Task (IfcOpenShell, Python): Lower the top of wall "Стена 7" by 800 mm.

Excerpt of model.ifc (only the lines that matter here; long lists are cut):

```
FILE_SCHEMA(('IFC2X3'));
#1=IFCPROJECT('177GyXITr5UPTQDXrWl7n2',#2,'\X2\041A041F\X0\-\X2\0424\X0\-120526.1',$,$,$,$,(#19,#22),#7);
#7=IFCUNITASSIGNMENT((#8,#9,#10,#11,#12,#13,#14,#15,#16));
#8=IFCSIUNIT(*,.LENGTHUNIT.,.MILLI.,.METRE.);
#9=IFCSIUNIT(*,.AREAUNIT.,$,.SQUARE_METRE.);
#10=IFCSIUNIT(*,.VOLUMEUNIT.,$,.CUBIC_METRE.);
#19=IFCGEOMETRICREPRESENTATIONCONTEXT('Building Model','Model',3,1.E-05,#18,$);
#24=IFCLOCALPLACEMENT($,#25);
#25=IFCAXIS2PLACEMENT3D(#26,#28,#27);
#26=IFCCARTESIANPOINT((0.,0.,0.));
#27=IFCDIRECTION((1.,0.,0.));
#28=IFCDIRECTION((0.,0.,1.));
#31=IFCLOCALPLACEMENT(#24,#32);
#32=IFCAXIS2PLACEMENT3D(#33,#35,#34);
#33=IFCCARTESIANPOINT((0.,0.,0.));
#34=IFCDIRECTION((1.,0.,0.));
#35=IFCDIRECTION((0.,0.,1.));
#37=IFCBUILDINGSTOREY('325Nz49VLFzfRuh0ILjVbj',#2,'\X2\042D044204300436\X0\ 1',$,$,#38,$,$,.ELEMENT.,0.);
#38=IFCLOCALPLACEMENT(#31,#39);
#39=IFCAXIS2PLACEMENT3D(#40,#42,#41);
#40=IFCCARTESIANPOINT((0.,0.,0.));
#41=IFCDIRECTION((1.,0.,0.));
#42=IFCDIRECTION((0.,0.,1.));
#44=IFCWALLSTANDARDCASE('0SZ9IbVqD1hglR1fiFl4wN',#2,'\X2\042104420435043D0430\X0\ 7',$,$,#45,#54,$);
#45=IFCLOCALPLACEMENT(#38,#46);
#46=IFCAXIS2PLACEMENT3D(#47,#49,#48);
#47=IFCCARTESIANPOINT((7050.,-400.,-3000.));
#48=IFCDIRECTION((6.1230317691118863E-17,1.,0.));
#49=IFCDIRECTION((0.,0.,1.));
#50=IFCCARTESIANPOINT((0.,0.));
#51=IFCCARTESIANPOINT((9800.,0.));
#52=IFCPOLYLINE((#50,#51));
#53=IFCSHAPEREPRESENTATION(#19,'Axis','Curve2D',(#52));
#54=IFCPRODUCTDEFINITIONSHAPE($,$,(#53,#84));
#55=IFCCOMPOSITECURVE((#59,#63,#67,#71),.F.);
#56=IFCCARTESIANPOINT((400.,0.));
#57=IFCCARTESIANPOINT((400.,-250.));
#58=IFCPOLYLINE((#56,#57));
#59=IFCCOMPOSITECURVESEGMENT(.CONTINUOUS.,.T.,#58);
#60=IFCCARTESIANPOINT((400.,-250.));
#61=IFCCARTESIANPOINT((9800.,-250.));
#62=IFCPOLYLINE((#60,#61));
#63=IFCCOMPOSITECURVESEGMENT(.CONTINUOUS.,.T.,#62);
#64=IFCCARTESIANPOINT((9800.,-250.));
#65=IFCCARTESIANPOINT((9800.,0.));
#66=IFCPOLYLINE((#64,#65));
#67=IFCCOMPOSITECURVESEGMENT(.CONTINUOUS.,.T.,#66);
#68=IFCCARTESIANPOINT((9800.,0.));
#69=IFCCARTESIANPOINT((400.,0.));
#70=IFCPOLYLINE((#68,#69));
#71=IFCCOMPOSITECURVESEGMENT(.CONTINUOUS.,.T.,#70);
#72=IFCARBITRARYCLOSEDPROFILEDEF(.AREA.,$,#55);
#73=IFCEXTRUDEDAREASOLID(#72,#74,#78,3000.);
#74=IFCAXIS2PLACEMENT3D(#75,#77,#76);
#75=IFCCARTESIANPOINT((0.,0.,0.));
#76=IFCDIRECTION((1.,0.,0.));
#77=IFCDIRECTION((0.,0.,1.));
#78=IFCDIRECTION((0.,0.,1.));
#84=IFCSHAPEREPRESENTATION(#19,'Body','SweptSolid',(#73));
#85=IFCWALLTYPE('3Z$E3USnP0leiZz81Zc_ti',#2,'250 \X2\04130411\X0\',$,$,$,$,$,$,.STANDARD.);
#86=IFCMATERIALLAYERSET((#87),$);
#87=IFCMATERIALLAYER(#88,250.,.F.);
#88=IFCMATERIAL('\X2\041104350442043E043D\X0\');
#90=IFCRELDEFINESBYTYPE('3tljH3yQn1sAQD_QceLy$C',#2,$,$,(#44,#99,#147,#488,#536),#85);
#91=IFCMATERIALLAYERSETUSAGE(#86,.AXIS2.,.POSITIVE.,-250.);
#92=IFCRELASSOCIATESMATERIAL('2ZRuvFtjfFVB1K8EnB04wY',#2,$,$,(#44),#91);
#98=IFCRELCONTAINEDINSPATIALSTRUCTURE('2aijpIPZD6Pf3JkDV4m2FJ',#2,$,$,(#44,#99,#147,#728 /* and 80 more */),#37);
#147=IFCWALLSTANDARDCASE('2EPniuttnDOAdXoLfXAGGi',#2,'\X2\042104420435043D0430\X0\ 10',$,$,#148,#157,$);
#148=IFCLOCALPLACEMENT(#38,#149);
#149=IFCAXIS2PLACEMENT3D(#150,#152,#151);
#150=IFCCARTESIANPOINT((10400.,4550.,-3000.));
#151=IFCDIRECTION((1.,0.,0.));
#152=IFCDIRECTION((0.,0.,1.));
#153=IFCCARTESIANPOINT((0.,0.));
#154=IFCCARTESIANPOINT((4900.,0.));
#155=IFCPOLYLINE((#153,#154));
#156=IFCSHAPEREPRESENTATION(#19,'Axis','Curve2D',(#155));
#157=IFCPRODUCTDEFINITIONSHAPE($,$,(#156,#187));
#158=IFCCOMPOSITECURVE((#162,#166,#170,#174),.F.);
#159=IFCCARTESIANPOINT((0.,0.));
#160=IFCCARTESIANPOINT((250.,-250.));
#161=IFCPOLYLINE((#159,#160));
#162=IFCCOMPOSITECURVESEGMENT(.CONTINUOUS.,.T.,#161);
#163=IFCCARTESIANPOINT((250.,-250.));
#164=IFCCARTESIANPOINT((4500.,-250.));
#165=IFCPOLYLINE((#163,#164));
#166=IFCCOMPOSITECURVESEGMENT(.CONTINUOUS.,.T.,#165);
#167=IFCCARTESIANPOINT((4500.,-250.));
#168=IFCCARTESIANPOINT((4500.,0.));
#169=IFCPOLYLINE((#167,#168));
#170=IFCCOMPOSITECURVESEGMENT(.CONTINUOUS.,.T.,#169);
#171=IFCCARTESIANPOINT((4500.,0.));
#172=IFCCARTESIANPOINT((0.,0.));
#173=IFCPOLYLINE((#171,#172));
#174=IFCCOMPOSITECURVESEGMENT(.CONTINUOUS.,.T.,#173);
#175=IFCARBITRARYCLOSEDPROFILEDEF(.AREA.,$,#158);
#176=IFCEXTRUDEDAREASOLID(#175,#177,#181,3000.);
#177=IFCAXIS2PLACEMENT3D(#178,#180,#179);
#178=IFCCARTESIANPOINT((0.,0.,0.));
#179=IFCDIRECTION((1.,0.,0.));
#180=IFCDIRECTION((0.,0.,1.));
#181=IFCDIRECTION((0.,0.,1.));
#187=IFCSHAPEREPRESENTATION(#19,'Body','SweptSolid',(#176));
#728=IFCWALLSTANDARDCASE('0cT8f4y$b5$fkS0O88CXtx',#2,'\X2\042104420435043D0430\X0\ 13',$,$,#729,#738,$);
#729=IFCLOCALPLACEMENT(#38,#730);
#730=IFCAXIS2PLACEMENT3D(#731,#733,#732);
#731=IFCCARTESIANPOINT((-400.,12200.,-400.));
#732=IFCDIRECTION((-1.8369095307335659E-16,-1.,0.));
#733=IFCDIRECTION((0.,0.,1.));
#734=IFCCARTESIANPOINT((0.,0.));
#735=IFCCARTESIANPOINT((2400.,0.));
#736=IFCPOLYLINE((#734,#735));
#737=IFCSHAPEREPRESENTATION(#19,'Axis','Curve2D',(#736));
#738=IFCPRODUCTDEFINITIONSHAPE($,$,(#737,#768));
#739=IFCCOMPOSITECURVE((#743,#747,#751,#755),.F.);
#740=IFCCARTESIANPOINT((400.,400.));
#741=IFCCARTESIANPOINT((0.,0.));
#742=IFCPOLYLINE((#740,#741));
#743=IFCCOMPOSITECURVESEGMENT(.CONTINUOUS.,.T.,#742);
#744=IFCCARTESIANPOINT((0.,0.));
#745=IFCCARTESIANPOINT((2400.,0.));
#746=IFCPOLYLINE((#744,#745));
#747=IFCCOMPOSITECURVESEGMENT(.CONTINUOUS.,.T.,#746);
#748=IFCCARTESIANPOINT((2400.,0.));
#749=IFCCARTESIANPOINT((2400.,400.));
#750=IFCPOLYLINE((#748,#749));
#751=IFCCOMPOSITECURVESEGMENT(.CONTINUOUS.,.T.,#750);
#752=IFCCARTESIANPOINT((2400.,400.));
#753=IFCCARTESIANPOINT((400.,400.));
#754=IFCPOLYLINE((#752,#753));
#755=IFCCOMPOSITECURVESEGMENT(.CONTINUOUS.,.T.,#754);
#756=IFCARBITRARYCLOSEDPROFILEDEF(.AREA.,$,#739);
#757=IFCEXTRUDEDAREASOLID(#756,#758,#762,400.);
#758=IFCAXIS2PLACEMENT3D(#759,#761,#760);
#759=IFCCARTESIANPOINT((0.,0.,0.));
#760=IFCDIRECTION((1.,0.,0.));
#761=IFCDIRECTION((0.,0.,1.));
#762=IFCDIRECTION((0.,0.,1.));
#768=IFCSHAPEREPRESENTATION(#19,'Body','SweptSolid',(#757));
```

```python
import ifcopenshell
import ifcopenshell.geom
import ifcopenshell.util.shape
import ifcopenshell.util.unit

model = ifcopenshell.open("model.ifc")
unit_scale = ifcopenshell.util.unit.calculate_unit_scale(model)
settings = ifcopenshell.geom.settings()


def volume(element):
    """Net volume in cubic metres, openings subtracted."""
    shape = ifcopenshell.geom.create_shape(settings, element)
    return ifcopenshell.util.shape.get_volume(shape.geometry)


wall = model.by_guid("0SZ9IbVqD1hglR1fiFl4wN")
before = volume(wall)

body = next(r for r in wall.Representation.Representations if r.RepresentationIdentifier == "Body")
solid = body.Items[0]
old_height = solid.Depth
solid.Depth -= 0.8 / unit_scale
after = volume(wall)

print(f"height {old_height:g} -> {solid.Depth:g}, volume {before:.3f} -> {after:.3f} m3")

model.write("model_updated.ifc")
```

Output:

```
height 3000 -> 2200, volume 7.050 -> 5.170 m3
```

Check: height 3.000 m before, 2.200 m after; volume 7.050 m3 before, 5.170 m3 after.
